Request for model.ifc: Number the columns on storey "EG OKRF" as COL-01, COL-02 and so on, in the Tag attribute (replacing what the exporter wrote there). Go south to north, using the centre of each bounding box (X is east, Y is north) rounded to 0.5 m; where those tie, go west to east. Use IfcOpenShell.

First a look at what the model holds.

```python
import ifcopenshell
import ifcopenshell.util.element
import ifcopenshell.util.placement

model = ifcopenshell.open("model.ifc")
print(model.schema)
storey = next(s for s in model.by_type("IfcBuildingStorey") if s.Name == "EG OKRF")
columns = [e for e in ifcopenshell.util.element.get_decomposition(storey) if e.is_a("IfcColumn")]
for e in sorted(columns, key=lambda e: e.id()):
    origin = ifcopenshell.util.placement.get_local_placement(e.ObjectPlacement)[:3, 3]
    print(e.id(), e.Tag, e.Name, origin.round(2) + 0.0, sep=" | ")
```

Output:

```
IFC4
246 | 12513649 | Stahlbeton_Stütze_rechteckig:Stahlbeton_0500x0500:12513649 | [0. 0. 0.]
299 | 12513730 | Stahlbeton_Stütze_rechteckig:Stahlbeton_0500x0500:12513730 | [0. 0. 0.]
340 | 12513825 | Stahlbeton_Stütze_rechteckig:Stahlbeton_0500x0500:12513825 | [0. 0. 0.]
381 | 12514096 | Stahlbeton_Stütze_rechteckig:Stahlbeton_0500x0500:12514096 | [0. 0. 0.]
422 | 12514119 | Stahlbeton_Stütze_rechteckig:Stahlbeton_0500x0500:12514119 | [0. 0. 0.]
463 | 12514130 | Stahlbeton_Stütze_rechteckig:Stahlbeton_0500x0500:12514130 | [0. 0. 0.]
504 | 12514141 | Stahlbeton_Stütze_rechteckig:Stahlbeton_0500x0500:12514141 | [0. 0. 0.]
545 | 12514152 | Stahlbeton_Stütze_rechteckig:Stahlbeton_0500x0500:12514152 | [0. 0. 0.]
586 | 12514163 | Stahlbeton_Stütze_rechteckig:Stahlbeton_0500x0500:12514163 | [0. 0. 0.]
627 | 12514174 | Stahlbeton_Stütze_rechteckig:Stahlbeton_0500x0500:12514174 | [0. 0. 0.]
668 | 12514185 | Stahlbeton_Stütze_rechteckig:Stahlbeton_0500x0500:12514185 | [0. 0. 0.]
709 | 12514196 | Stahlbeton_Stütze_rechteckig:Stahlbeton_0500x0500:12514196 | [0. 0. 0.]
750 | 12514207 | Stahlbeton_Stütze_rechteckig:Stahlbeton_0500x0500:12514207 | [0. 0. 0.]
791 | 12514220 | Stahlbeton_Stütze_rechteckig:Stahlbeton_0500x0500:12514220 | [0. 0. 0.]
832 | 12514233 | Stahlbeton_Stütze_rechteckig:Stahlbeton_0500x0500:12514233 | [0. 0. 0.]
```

```python
import ifcopenshell
import ifcopenshell.geom
import ifcopenshell.util.element
import ifcopenshell.util.shape

model = ifcopenshell.open("model.ifc")
settings = ifcopenshell.geom.settings()
settings.set("use-world-coords", True)


def centre(element):
    shape = ifcopenshell.geom.create_shape(settings, element)
    return ifcopenshell.util.shape.get_bbox_centroid(shape.geometry)


storey = next(s for s in model.by_type("IfcBuildingStorey") if s.Name == "EG OKRF")
columns = [e for e in ifcopenshell.util.element.get_decomposition(storey) if e.is_a("IfcColumn")]

# Insertion points can sit at a corner or the storey origin, so sort by the geometry (in metres).
centres = {e: centre(e) for e in columns}
columns.sort(key=lambda e: (round(centres[e][1] / 0.5), centres[e][0]))

for i, e in enumerate(columns, start=1):
    number = f"COL-{i:02d}"
    e.Tag = number
    print(e.id(), number)

model.write("model_updated.ifc")
```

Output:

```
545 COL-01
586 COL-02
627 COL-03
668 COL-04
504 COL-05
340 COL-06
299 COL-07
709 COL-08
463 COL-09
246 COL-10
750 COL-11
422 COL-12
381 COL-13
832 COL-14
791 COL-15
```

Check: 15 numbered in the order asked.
